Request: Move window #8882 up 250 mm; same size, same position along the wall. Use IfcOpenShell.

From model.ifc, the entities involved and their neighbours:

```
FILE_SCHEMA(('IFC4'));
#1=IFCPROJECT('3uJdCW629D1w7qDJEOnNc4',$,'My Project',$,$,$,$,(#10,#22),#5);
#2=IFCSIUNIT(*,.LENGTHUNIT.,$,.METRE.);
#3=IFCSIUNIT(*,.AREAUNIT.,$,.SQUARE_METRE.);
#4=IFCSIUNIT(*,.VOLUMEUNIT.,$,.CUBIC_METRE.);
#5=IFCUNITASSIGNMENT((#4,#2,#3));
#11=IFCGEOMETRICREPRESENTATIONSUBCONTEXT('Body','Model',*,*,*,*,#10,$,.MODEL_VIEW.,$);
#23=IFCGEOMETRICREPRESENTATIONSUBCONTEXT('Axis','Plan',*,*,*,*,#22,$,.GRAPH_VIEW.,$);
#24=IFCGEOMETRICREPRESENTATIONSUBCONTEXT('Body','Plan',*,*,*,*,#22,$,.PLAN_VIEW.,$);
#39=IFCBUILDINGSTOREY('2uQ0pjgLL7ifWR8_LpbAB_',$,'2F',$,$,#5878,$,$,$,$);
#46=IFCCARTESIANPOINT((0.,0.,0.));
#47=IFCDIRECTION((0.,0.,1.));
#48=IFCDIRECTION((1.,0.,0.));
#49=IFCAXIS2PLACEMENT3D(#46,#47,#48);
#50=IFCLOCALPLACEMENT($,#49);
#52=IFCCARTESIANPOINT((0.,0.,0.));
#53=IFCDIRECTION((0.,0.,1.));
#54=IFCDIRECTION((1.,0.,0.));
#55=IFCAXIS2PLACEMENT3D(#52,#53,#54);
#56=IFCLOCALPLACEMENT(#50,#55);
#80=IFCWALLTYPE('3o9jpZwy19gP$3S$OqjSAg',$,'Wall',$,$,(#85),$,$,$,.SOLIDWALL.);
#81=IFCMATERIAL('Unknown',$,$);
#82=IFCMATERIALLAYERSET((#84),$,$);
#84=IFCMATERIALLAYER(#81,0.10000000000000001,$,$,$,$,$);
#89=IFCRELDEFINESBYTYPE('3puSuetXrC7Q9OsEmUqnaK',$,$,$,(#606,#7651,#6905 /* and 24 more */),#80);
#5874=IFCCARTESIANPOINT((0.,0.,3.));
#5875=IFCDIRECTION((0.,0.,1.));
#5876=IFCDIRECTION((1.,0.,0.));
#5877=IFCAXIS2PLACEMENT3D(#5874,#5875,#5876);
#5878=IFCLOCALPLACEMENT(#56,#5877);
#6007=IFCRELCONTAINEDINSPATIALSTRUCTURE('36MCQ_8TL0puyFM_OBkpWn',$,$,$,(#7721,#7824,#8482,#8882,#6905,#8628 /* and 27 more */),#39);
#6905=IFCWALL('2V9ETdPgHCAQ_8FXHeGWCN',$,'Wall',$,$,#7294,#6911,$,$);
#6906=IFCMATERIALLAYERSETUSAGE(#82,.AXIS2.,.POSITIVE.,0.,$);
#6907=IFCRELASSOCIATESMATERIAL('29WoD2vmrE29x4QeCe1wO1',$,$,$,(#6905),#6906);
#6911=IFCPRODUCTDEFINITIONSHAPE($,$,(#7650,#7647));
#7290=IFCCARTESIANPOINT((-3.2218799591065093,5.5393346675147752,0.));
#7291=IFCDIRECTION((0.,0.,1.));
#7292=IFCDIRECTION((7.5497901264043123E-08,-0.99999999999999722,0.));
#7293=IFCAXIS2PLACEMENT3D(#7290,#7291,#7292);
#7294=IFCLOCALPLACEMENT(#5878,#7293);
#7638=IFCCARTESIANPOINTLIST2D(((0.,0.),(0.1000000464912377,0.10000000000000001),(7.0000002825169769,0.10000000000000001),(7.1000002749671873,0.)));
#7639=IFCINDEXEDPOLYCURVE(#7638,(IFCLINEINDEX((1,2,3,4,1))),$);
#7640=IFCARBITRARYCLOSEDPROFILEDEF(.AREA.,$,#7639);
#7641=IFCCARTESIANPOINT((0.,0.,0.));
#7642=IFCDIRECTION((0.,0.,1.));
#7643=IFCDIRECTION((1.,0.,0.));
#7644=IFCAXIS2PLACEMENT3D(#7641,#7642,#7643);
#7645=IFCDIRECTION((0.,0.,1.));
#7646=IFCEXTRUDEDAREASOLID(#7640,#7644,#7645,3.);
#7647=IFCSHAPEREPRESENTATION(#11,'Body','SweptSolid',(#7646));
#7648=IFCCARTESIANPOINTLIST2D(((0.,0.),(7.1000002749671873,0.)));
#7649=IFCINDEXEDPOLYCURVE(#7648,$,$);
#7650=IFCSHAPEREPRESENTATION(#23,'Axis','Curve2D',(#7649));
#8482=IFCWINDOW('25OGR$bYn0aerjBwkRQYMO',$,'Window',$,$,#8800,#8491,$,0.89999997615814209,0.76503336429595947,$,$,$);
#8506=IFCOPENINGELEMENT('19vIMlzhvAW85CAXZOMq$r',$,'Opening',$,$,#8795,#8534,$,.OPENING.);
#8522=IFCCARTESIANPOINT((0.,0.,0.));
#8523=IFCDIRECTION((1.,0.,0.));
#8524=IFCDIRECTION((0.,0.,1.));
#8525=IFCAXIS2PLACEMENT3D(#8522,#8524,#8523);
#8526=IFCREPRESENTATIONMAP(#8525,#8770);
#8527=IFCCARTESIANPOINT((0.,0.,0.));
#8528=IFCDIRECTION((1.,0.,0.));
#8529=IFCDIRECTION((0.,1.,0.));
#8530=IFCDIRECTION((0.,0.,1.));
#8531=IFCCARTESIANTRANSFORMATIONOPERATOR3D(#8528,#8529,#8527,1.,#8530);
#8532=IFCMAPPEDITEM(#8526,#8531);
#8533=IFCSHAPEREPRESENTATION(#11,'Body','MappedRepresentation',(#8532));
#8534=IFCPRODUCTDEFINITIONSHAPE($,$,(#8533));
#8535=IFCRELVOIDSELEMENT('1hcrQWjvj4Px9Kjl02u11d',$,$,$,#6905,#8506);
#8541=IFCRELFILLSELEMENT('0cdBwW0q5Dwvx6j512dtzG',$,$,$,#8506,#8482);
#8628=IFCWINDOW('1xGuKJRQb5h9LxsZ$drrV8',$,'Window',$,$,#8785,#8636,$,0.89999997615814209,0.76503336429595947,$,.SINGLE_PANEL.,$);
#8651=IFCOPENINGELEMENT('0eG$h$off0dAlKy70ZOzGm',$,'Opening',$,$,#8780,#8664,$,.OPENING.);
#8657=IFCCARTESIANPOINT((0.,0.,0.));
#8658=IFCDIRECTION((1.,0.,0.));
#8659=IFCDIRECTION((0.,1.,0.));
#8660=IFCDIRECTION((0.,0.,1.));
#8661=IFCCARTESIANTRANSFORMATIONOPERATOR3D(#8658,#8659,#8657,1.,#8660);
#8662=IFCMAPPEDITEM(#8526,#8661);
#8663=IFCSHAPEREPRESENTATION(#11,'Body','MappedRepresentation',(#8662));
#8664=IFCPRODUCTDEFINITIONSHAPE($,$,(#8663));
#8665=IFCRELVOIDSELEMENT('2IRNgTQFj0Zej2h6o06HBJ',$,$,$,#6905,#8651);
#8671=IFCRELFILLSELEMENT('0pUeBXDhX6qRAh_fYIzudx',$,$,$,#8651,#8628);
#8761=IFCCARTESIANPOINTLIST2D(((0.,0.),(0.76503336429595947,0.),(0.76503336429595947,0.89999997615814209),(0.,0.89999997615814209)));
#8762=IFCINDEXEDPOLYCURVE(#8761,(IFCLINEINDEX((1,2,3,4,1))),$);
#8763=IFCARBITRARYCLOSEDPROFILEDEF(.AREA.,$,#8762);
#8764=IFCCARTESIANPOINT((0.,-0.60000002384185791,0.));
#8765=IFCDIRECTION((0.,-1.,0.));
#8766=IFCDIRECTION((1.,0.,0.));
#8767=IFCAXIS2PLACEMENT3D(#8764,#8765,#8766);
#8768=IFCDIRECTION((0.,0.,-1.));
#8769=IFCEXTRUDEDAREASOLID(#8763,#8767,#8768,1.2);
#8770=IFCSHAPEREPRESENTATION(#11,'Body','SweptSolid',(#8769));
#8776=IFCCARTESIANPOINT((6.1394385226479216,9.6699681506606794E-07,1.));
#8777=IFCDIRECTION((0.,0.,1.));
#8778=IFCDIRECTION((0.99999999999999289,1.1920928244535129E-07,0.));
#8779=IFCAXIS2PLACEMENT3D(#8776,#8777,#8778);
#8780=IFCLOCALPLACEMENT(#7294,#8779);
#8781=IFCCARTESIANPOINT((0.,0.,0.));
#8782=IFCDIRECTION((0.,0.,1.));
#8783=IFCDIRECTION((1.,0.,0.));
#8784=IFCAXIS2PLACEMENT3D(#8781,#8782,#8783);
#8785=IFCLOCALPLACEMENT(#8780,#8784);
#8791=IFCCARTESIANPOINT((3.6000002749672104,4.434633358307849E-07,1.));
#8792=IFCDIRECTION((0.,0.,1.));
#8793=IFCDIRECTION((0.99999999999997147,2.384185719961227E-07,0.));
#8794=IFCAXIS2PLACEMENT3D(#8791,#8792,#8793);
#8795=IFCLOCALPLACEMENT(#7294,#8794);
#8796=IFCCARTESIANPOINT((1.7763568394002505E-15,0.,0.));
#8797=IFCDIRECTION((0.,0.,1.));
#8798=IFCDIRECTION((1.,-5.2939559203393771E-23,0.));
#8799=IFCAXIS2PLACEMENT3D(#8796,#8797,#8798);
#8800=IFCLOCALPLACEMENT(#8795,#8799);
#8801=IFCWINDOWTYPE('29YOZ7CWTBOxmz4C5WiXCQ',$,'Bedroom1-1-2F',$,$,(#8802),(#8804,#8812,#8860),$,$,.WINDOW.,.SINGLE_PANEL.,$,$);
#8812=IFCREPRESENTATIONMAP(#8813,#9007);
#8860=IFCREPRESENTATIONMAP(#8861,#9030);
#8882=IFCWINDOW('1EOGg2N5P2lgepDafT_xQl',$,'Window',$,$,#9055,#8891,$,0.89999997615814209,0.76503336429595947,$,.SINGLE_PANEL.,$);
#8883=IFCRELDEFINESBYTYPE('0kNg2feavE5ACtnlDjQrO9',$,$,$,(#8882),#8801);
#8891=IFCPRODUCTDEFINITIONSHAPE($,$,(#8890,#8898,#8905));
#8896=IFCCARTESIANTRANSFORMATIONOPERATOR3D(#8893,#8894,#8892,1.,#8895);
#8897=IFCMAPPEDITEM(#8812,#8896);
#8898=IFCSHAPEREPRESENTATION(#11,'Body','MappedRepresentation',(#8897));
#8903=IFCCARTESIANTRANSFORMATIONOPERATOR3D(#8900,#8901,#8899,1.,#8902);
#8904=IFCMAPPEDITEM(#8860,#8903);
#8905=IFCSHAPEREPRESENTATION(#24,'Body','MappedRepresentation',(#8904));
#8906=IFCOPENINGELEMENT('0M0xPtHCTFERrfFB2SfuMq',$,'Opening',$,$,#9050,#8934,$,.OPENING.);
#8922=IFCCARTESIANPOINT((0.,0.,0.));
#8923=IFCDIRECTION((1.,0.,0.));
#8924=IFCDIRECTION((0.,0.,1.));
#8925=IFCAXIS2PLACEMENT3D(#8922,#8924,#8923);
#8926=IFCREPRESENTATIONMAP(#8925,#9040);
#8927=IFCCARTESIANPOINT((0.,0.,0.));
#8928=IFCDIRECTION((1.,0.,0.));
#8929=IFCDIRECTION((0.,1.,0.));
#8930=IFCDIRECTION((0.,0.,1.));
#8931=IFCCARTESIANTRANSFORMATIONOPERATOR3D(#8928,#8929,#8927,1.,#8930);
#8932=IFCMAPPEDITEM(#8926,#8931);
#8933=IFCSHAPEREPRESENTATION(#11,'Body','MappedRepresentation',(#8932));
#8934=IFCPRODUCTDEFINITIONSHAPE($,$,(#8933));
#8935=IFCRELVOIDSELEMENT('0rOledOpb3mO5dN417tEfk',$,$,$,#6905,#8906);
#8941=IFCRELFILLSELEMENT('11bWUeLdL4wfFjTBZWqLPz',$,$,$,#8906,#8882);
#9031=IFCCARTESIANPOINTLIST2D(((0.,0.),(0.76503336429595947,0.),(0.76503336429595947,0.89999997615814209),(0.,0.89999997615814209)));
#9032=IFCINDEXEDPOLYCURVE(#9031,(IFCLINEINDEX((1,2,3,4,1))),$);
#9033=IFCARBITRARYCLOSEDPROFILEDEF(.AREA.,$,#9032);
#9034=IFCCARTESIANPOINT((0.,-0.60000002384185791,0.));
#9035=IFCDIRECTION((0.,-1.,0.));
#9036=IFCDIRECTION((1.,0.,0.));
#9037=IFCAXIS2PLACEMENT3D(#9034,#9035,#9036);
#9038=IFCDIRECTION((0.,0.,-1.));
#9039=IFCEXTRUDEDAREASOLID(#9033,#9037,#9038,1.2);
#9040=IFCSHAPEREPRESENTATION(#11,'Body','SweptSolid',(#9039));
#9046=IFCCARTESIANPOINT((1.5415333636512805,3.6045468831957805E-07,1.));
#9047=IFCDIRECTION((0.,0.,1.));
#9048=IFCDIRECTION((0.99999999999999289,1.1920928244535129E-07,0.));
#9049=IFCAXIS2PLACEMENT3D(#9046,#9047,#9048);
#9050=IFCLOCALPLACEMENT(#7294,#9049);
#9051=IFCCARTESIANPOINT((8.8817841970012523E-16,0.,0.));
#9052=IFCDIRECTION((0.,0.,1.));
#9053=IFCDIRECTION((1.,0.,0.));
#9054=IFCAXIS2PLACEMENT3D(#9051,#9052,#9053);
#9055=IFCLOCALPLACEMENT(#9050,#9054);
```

```python
import numpy as np
import ifcopenshell
import ifcopenshell.api.geometry
import ifcopenshell.util.placement
import ifcopenshell.util.unit

model = ifcopenshell.open("model.ifc")
unit_scale = ifcopenshell.util.unit.calculate_unit_scale(model)

window = model.by_guid("1EOGg2N5P2lgepDafT_xQl")
opening = window.FillsVoids[0].RelatingOpeningElement
dz = 0.25

shift = np.array([0.0, 0.0, dz])
# The window is placed relative to its opening, so it follows when the opening moves.
matrix = ifcopenshell.util.placement.get_local_placement(opening.ObjectPlacement)
matrix[:3, 3] += shift
ifcopenshell.api.geometry.edit_object_placement(
    model, product=opening, matrix=matrix, is_si=False, should_transform_children=True
)

print(f"moved by {dz * unit_scale:+.3f} m")

model.write("model-out.ifc")
```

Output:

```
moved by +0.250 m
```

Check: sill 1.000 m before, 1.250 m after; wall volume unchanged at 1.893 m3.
